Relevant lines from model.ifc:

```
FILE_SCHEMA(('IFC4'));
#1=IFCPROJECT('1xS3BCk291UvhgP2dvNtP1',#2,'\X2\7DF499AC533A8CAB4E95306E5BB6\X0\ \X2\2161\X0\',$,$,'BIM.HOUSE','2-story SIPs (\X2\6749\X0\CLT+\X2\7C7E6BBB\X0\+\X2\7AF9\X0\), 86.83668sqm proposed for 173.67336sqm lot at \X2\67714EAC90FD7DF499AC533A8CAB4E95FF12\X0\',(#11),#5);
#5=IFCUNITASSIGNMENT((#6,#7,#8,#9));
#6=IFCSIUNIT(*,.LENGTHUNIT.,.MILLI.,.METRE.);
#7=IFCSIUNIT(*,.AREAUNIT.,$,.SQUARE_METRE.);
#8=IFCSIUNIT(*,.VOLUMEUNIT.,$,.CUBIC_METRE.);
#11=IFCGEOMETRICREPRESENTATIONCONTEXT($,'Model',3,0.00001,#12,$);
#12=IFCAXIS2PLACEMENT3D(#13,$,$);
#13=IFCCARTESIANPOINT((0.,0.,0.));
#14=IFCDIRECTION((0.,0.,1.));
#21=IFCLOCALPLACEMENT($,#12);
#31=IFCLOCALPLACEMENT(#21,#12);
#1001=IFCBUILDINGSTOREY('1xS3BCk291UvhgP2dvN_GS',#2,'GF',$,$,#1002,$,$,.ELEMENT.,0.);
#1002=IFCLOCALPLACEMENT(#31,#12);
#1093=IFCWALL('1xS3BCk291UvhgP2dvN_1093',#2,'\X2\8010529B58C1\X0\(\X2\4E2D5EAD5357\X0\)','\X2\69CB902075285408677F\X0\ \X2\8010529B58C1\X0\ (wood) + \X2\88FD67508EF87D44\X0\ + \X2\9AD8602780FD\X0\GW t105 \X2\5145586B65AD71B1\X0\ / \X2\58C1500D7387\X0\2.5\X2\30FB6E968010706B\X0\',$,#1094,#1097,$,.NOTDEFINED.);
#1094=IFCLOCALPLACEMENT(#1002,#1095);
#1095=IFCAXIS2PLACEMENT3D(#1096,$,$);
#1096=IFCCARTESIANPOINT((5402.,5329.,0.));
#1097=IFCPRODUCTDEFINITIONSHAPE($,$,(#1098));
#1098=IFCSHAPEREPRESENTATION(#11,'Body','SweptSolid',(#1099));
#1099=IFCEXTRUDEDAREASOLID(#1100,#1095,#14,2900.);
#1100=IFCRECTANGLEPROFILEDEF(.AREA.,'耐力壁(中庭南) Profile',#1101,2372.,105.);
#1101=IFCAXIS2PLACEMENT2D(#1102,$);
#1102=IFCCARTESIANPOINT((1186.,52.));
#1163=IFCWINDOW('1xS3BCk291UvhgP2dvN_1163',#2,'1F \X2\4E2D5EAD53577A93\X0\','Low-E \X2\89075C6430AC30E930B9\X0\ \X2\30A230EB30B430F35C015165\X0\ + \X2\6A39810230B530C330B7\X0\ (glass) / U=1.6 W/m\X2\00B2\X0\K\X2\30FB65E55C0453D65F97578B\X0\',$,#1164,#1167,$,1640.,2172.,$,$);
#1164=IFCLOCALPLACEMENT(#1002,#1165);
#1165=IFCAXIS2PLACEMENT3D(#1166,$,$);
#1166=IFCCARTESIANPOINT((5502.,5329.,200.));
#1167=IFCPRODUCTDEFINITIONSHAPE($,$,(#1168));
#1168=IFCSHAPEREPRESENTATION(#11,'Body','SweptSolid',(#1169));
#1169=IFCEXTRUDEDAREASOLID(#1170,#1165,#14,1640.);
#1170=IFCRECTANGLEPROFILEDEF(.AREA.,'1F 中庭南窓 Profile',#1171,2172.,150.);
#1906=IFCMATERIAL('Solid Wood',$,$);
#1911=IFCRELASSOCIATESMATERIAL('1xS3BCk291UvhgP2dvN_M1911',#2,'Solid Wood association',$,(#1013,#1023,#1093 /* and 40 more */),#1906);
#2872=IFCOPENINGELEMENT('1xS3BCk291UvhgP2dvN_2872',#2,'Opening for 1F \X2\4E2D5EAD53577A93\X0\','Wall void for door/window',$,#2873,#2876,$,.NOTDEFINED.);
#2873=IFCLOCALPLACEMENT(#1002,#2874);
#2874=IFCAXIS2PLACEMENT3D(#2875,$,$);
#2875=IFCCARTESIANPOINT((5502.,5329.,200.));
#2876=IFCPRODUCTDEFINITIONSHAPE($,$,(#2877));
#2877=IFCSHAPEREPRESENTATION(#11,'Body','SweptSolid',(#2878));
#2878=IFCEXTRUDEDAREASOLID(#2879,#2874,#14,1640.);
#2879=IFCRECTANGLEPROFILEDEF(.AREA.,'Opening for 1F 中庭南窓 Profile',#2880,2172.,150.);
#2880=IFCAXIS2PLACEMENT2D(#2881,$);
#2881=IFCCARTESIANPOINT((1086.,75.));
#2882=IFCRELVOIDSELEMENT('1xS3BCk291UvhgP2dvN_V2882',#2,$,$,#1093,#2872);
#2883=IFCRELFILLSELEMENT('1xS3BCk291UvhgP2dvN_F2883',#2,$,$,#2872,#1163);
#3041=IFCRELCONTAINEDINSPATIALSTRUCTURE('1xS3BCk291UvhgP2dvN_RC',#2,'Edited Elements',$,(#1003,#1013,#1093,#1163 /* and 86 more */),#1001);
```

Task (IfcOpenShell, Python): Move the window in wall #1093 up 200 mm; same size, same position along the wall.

```python
import numpy as np
import ifcopenshell
import ifcopenshell.api.geometry
import ifcopenshell.util.placement
import ifcopenshell.util.unit

model = ifcopenshell.open("model.ifc")
unit_scale = ifcopenshell.util.unit.calculate_unit_scale(model)

window = model.by_guid("1xS3BCk291UvhgP2dvN_1163")
opening = window.FillsVoids[0].RelatingOpeningElement
dz = 0.2 / unit_scale

shift = np.array([0.0, 0.0, dz])
# The window is not placed relative to its opening, so move both.
for product in (opening, window):
    matrix = ifcopenshell.util.placement.get_local_placement(product.ObjectPlacement)
    matrix[:3, 3] += shift
    ifcopenshell.api.geometry.edit_object_placement(model, product=product, matrix=matrix, is_si=False)

print(f"moved by {dz * unit_scale:+.3f} m")

model.write("model_updated.ifc")
```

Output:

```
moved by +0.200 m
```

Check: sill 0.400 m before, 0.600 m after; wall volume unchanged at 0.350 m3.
